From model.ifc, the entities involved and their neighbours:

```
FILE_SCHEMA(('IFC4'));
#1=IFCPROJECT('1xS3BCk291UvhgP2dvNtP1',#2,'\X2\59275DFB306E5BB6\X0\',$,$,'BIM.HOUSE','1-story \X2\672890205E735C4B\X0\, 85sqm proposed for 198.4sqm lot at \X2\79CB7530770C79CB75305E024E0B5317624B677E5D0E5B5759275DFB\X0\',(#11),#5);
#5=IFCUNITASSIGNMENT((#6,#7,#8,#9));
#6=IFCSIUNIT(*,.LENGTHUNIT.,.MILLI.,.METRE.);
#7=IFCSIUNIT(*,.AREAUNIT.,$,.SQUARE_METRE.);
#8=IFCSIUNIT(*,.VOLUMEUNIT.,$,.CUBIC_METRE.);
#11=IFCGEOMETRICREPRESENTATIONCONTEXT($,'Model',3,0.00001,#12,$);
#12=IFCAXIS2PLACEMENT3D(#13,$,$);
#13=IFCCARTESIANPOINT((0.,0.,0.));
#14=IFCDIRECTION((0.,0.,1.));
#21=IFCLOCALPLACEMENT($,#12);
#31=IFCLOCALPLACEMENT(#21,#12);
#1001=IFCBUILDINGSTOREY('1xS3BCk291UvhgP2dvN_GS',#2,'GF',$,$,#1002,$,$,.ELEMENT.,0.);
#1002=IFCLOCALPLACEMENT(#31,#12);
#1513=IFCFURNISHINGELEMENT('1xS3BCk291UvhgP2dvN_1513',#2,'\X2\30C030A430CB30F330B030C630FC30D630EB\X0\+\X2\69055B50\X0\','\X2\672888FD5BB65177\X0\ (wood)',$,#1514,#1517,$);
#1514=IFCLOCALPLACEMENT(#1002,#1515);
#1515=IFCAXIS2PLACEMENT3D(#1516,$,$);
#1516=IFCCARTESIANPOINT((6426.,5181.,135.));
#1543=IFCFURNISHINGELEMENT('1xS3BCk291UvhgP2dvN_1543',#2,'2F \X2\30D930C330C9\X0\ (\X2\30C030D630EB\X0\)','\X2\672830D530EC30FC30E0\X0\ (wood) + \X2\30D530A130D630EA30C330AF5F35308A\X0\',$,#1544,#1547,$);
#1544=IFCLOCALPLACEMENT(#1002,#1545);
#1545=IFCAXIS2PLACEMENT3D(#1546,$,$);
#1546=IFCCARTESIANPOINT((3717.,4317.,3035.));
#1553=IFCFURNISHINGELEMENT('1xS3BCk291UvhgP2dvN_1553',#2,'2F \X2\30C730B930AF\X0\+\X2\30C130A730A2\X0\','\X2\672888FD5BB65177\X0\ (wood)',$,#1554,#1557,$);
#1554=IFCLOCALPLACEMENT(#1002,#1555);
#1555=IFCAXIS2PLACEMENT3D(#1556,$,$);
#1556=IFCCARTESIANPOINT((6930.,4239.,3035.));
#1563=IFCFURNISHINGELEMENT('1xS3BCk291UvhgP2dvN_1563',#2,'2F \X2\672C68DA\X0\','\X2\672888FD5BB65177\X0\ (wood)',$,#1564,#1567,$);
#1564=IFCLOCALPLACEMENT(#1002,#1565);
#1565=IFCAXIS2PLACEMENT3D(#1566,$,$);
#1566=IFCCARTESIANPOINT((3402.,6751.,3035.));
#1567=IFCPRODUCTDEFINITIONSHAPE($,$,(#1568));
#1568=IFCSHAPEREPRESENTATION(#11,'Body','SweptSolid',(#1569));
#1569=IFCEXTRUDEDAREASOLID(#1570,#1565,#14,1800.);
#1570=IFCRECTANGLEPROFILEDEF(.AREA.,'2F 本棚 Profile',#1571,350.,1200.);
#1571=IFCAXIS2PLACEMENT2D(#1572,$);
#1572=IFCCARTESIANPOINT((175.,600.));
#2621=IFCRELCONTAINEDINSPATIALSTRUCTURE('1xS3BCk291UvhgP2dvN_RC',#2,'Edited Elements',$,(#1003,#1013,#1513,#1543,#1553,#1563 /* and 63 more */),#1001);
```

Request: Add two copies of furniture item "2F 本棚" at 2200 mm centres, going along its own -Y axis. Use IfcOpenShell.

```python
import ifcopenshell
import ifcopenshell.api.geometry
import ifcopenshell.api.root
import ifcopenshell.util.element
import ifcopenshell.util.placement

model = ifcopenshell.open("model.ifc")


def reuse_history(source, copy):
    """copy_class also copies each property set's owner history, people and application; keep the originals."""
    for rel in copy.IsDefinedBy:
        if rel.is_a("IfcRelDefinesByProperties") and (history := rel.RelatingPropertyDefinition.OwnerHistory):
            rel.RelatingPropertyDefinition.OwnerHistory = source.OwnerHistory
            ifcopenshell.util.element.remove_deep2(model, history)


source = model.by_guid("1xS3BCk291UvhgP2dvN_1563")
base = ifcopenshell.util.placement.get_local_placement(source.ObjectPlacement)
step = -base[:3, 1] * 2200.0

for i in range(1, 3):
    copy = ifcopenshell.api.root.copy_class(model, product=source)
    copy.Representation = ifcopenshell.util.element.copy_deep(
        model, source.Representation, exclude=["IfcGeometricRepresentationContext", "IfcRepresentationMap"]
    )
    reuse_history(source, copy)
    matrix = base.copy()
    matrix[:3, 3] += i * step
    print("added at", matrix[:3, 3].round(3) + 0.0)
    ifcopenshell.api.geometry.edit_object_placement(model, product=copy, matrix=matrix, is_si=False)

model.write("model-out.ifc")
```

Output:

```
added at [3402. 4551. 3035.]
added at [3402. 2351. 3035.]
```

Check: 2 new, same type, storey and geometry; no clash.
